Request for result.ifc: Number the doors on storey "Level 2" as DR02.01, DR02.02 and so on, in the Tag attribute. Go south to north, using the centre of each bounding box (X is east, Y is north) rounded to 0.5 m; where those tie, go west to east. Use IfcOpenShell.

First a look at what the model holds.

```python
import ifcopenshell
import ifcopenshell.util.element
import ifcopenshell.util.placement

model = ifcopenshell.open("result.ifc")
print(model.schema)
storey = next(s for s in model.by_type("IfcBuildingStorey") if s.Name == "Level 2")
doors = [e for e in ifcopenshell.util.element.get_decomposition(storey) if e.is_a("IfcDoor")]
for e in sorted(doors, key=lambda e: e.id()):
    origin = ifcopenshell.util.placement.get_local_placement(e.ObjectPlacement)[:3, 3]
    print(e.id(), e.Tag, e.Name, origin.round(2) + 0.0, sep=" | ")
```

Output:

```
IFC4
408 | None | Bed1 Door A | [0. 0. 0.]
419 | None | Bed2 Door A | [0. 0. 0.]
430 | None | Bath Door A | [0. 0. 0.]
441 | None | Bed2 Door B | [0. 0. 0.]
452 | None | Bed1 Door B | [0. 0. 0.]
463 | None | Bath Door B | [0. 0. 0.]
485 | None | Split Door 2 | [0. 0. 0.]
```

```python
import ifcopenshell
import ifcopenshell.geom
import ifcopenshell.util.element
import ifcopenshell.util.shape

model = ifcopenshell.open("result.ifc")
settings = ifcopenshell.geom.settings()
settings.set("use-world-coords", True)


def centre(element):
    shape = ifcopenshell.geom.create_shape(settings, element)
    return ifcopenshell.util.shape.get_bbox_centroid(shape.geometry)


storey = next(s for s in model.by_type("IfcBuildingStorey") if s.Name == "Level 2")
doors = [e for e in ifcopenshell.util.element.get_decomposition(storey) if e.is_a("IfcDoor")]

# Insertion points can sit at a corner or the storey origin, so sort by the geometry (in metres).
centres = {e: centre(e) for e in doors}
doors.sort(key=lambda e: (round(centres[e][1] / 0.5), centres[e][0]))

for i, e in enumerate(doors, start=1):
    number = f"DR02.{i:02d}"
    e.Tag = number
    print(e.id(), number)

model.write("result-out.ifc")
```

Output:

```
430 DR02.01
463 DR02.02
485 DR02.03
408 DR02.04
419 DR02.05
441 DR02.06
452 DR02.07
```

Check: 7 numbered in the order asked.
